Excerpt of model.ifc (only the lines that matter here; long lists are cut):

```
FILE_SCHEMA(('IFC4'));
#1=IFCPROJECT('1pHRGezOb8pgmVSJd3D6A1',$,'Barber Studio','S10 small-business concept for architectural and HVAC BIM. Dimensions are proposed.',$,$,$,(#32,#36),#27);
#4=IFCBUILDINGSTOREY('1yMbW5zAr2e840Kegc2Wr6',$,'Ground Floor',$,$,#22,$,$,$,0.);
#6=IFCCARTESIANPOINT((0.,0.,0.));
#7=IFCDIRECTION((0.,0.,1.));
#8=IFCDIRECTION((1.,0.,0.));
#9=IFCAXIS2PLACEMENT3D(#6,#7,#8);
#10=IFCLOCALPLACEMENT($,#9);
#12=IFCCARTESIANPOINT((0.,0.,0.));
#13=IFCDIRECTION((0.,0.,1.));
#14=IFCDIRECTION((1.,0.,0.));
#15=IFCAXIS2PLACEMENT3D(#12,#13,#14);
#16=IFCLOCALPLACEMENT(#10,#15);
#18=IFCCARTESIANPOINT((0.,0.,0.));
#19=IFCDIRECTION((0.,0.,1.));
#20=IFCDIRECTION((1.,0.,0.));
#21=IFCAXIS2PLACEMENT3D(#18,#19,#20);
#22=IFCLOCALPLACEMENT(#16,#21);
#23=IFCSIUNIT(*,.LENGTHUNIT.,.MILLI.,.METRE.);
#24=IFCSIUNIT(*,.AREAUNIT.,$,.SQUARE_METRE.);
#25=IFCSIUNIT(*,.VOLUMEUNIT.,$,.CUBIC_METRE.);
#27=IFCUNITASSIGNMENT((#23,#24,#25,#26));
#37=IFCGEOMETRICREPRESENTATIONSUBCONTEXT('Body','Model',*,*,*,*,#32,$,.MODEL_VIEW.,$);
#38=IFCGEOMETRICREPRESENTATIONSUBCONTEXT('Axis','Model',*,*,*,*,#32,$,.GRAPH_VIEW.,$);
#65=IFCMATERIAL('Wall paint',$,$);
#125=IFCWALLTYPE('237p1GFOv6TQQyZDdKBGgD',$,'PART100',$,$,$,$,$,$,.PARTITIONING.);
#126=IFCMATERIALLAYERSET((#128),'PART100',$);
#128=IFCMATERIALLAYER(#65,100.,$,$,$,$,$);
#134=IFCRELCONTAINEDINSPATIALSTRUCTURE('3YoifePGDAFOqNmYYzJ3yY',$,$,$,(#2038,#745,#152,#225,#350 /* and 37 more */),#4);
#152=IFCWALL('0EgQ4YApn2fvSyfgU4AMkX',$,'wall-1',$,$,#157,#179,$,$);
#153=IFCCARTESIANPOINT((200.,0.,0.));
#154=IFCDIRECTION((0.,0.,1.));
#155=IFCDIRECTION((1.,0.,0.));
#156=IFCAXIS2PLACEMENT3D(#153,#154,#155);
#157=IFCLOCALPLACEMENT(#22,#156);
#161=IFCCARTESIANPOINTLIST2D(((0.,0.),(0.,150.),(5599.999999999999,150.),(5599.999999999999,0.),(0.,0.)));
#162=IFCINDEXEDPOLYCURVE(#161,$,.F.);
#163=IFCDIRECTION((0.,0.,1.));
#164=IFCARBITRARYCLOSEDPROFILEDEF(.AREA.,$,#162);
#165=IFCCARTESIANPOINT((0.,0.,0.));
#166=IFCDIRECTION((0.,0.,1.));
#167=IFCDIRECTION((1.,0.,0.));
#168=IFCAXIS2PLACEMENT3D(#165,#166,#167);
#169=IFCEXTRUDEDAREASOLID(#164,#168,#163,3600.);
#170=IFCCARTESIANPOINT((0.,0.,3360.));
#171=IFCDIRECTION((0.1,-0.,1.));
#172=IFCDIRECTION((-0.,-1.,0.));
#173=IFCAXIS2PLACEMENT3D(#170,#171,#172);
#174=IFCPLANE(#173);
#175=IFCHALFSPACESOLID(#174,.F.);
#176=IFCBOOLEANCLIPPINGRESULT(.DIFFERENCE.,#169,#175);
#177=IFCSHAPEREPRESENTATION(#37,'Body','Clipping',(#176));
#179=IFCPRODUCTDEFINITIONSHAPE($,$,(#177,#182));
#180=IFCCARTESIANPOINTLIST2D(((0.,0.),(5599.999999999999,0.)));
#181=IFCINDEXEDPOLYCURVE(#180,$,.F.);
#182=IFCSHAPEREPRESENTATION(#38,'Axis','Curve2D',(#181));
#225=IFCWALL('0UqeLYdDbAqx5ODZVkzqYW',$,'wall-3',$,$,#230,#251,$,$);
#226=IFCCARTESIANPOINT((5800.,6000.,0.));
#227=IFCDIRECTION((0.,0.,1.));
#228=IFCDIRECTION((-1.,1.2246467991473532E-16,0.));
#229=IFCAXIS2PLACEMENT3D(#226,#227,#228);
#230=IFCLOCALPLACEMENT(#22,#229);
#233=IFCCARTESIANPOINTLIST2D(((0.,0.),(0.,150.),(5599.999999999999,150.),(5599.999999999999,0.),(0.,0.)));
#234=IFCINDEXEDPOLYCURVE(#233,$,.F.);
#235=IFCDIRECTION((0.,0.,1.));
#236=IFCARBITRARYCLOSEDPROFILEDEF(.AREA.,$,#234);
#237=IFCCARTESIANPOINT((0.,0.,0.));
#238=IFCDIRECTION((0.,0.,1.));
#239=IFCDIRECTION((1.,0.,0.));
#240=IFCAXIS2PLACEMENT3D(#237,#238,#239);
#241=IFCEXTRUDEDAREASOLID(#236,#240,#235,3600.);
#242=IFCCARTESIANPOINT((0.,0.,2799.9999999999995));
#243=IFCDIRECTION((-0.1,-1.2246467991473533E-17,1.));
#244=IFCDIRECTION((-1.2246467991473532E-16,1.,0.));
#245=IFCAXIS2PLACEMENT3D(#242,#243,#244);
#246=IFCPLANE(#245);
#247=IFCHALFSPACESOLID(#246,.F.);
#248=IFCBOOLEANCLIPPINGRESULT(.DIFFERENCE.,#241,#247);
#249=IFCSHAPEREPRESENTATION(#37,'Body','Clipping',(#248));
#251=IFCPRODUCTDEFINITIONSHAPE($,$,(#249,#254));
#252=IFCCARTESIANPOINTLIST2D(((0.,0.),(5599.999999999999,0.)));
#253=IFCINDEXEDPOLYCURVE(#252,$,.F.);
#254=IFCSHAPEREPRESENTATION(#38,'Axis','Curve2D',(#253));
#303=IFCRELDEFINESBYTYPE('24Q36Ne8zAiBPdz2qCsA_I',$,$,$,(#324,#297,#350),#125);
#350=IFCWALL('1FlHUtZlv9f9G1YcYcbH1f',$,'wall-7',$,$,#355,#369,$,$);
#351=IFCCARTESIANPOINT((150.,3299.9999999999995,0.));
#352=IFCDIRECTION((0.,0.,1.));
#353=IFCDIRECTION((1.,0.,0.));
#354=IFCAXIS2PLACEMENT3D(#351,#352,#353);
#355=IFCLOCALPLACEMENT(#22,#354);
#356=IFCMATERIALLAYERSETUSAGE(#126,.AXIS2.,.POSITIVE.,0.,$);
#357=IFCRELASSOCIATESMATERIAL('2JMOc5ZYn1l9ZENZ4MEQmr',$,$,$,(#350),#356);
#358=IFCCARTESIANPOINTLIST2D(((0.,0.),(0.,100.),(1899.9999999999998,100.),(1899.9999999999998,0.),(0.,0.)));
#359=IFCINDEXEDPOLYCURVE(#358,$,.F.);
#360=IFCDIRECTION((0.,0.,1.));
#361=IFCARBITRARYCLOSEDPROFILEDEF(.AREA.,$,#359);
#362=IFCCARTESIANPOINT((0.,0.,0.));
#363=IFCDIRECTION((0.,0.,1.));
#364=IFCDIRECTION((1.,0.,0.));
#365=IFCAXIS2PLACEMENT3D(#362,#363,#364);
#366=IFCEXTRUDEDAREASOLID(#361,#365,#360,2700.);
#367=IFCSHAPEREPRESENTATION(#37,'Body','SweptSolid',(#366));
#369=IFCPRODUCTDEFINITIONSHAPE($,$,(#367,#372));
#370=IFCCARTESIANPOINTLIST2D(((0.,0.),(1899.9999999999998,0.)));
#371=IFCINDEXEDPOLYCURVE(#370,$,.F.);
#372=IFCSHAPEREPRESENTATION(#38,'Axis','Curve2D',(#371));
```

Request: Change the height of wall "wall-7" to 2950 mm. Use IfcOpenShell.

```python
import ifcopenshell
import ifcopenshell.geom
import ifcopenshell.util.representation
import ifcopenshell.util.shape
import ifcopenshell.util.unit

model = ifcopenshell.open("model.ifc")
unit_scale = ifcopenshell.util.unit.calculate_unit_scale(model)
settings = ifcopenshell.geom.settings()


def volume(element):
    """Net volume in cubic metres, openings subtracted."""
    shape = ifcopenshell.geom.create_shape(settings, element)
    return ifcopenshell.util.shape.get_volume(shape.geometry)


wall = model.by_guid("1FlHUtZlv9f9G1YcYcbH1f")
before = volume(wall)

body = ifcopenshell.util.representation.get_representation(wall, "Model", "Body")
solid = body.Items[0]
old_height = solid.Depth
solid.Depth = 2.95 / unit_scale
after = volume(wall)

print(f"height {old_height:g} -> {solid.Depth:g}, volume {before:.3f} -> {after:.3f} m3")

model.write("model_v2.ifc")
```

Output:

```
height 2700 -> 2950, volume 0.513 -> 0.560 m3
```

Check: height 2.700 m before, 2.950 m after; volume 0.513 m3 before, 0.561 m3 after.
